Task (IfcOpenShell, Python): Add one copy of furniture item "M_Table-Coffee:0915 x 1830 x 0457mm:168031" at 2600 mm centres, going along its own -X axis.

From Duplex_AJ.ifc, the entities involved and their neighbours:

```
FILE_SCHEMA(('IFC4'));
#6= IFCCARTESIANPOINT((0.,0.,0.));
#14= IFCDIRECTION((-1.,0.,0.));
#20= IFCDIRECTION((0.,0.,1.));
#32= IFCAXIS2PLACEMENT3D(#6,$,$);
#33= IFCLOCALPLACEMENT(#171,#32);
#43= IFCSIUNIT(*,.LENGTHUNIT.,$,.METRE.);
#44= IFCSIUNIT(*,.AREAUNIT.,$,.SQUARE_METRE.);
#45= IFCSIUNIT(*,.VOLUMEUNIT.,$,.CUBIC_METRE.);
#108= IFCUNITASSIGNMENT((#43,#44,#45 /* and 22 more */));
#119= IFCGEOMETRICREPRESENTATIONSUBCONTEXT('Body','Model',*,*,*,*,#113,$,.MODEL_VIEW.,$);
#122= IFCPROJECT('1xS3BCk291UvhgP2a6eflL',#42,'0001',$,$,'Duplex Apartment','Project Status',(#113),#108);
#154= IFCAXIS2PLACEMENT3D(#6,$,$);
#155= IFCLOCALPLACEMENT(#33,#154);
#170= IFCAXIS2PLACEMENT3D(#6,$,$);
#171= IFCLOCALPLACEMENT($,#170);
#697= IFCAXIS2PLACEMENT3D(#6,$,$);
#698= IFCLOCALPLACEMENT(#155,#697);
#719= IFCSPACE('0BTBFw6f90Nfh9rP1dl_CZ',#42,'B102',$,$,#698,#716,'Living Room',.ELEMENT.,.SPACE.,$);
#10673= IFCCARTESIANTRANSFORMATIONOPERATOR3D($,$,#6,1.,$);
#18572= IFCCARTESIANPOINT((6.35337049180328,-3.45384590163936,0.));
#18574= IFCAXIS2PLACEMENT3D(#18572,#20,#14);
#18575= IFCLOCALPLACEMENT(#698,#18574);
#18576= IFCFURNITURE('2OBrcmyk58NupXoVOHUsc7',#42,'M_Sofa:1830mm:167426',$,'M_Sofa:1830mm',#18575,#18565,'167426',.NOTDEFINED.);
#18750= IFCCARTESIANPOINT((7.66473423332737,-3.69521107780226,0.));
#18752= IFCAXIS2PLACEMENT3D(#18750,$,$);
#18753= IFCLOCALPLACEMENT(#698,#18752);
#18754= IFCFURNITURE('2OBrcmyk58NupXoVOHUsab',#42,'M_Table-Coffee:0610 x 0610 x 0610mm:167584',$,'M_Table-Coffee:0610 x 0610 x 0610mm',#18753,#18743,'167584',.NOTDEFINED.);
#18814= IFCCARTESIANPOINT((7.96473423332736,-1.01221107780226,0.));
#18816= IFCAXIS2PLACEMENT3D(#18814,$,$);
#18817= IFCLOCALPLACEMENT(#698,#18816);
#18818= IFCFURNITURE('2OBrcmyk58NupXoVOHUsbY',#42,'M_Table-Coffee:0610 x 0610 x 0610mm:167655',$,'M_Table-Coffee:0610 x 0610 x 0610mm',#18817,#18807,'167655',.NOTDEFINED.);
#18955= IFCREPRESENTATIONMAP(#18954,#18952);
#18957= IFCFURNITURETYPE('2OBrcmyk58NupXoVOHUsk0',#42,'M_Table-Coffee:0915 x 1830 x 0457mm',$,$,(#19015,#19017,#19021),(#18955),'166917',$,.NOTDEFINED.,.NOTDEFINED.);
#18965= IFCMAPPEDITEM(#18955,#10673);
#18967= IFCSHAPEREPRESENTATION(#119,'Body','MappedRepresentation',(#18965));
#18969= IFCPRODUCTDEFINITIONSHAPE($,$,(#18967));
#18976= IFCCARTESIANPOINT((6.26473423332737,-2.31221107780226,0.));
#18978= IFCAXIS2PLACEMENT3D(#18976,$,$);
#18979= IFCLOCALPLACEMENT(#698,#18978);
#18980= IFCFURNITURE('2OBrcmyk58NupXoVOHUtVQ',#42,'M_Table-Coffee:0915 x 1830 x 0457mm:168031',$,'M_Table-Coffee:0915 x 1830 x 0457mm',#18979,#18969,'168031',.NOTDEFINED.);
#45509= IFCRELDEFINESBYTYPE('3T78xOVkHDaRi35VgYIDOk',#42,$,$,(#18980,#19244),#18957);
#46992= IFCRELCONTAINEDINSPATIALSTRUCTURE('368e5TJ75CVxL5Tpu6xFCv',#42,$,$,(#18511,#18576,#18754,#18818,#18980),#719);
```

```python
import ifcopenshell
import ifcopenshell.api.geometry
import ifcopenshell.api.root
import ifcopenshell.util.element
import ifcopenshell.util.placement
import ifcopenshell.util.unit

model = ifcopenshell.open("Duplex_AJ.ifc")
unit_scale = ifcopenshell.util.unit.calculate_unit_scale(model)


def reuse_history(source, copy):
    """copy_class also copies each property set's owner history, people and application; keep the originals."""
    for rel in copy.IsDefinedBy:
        if rel.is_a("IfcRelDefinesByProperties") and (history := rel.RelatingPropertyDefinition.OwnerHistory):
            rel.RelatingPropertyDefinition.OwnerHistory = source.OwnerHistory
            ifcopenshell.util.element.remove_deep2(model, history)


source = model.by_guid("2OBrcmyk58NupXoVOHUtVQ")
base = ifcopenshell.util.placement.get_local_placement(source.ObjectPlacement)
step = -base[:3, 0] * 2.6 / unit_scale

for i in range(1, 2):
    copy = ifcopenshell.api.root.copy_class(model, product=source)
    copy.Representation = ifcopenshell.util.element.copy_deep(
        model, source.Representation, exclude=["IfcGeometricRepresentationContext", "IfcRepresentationMap"]
    )
    copy.Name = "M_Table-Coffee:0915 x 1830 x 0457mm"
    copy.Tag = None
    reuse_history(source, copy)
    matrix = base.copy()
    matrix[:3, 3] += i * step
    print("added at", matrix[:3, 3].round(3) + 0.0)
    ifcopenshell.api.geometry.edit_object_placement(model, product=copy, matrix=matrix, is_si=False)

model.write("Duplex_AJ_v2.ifc")
```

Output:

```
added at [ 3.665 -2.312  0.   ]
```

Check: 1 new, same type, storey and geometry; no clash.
